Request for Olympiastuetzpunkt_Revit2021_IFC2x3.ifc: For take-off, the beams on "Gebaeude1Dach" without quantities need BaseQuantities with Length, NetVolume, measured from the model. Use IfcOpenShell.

First a look at what the model holds.

```python
import ifcopenshell
import ifcopenshell.util.element
import ifcopenshell.util.unit

model = ifcopenshell.open("Olympiastuetzpunkt_Revit2021_IFC2x3.ifc")
print(model.schema)
for unit_type in ("LENGTHUNIT", "AREAUNIT", "VOLUMEUNIT"):
    print(unit_type, ifcopenshell.util.unit.calculate_unit_scale(model, unit_type))
storey = next(s for s in model.by_type("IfcBuildingStorey") if s.Name == "Gebaeude1Dach")
beams = [e for e in ifcopenshell.util.element.get_decomposition(storey) if e.is_a("IfcBeam")]
for e in sorted(beams, key=lambda e: e.id()):
    print(e.id(), e.is_a(), e.Name, list(ifcopenshell.util.element.get_psets(e, qtos_only=True)), sep=" | ")
```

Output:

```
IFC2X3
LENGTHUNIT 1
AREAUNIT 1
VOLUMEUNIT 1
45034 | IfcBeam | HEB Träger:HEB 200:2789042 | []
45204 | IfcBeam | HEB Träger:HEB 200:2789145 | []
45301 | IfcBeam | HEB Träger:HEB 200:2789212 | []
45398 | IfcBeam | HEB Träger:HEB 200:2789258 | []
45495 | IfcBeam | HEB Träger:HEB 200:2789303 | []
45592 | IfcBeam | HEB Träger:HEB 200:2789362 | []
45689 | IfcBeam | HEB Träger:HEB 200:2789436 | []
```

```python
import ifcopenshell
import ifcopenshell.api.pset
import ifcopenshell.geom
import ifcopenshell.util.element
import ifcopenshell.util.shape
import ifcopenshell.util.unit

model = ifcopenshell.open("Olympiastuetzpunkt_Revit2021_IFC2x3.ifc")
unit_scale = ifcopenshell.util.unit.calculate_unit_scale(model)
volume_scale = ifcopenshell.util.unit.calculate_unit_scale(model, "VOLUMEUNIT")
settings = ifcopenshell.geom.settings()

storey = next(s for s in model.by_type("IfcBuildingStorey") if s.Name == "Gebaeude1Dach")
beams = [e for e in ifcopenshell.util.element.get_decomposition(storey) if e.is_a("IfcBeam")]

for e in sorted(beams, key=lambda e: e.id()):
    if ifcopenshell.util.element.get_psets(e, qtos_only=True, should_inherit=False):
        continue
    # Geometry comes back in metres, in the element's own axes.
    shape = ifcopenshell.geom.create_shape(settings, e)
    values = {
        "Length": ifcopenshell.util.shape.get_max_xyz(shape.geometry) / unit_scale,
        "NetVolume": ifcopenshell.util.shape.get_volume(shape.geometry) / volume_scale,
    }
    qto = ifcopenshell.api.pset.add_qto(model, product=e, name="BaseQuantities")
    ifcopenshell.api.pset.edit_qto(model, qto=qto, properties=values)
    print(e.id(), {k: round(v, 3) for k, v in values.items()})

model.write("Olympiastuetzpunkt_Revit2021_IFC2x3_rev.ifc")
```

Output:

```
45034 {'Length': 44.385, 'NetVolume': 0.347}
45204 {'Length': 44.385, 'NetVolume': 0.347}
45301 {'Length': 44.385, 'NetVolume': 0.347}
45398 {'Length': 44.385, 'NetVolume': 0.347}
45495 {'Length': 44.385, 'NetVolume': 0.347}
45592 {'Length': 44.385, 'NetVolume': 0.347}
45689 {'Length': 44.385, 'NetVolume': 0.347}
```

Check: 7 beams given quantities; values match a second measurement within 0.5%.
